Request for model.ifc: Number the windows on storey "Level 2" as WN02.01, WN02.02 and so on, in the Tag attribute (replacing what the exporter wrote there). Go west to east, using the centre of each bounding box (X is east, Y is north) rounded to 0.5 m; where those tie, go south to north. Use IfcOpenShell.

First a look at what the model holds.

```python
import ifcopenshell
import ifcopenshell.util.element
import ifcopenshell.util.placement

model = ifcopenshell.open("model.ifc")
print(model.schema)
storey = next(s for s in model.by_type("IfcBuildingStorey") if s.Name == "Level 2")
windows = [e for e in ifcopenshell.util.element.get_decomposition(storey) if e.is_a("IfcWindow")]
for e in sorted(windows, key=lambda e: e.id()):
    origin = ifcopenshell.util.placement.get_local_placement(e.ObjectPlacement)[:3, 3]
    print(e.id(), e.Tag, e.Name, origin.round(2) + 0.0, sep=" | ")
```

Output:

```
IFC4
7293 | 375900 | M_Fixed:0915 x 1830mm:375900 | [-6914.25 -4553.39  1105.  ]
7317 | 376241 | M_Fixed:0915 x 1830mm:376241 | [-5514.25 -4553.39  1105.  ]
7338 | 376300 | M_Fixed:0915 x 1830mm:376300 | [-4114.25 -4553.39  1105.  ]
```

```python
import ifcopenshell
import ifcopenshell.geom
import ifcopenshell.util.element
import ifcopenshell.util.shape

model = ifcopenshell.open("model.ifc")
settings = ifcopenshell.geom.settings()
settings.set("use-world-coords", True)


def centre(element):
    shape = ifcopenshell.geom.create_shape(settings, element)
    return ifcopenshell.util.shape.get_bbox_centroid(shape.geometry)


storey = next(s for s in model.by_type("IfcBuildingStorey") if s.Name == "Level 2")
windows = [e for e in ifcopenshell.util.element.get_decomposition(storey) if e.is_a("IfcWindow")]

# Insertion points can sit at a corner or the storey origin, so sort by the geometry (in metres).
centres = {e: centre(e) for e in windows}
windows.sort(key=lambda e: (round(centres[e][0] / 0.5), centres[e][1]))

for i, e in enumerate(windows, start=1):
    number = f"WN02.{i:02d}"
    e.Tag = number
    print(e.id(), number)

model.write("model_updated.ifc")
```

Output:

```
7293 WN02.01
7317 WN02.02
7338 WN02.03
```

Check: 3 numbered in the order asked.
